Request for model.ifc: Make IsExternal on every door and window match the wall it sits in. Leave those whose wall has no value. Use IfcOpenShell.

First a look at what the model holds.

```python
import ifcopenshell
import ifcopenshell.util.element

model = ifcopenshell.open("model.ifc")
print(model.schema)
seen = {}
for e in model.by_type("IfcDoor") + model.by_type("IfcWindow"):
    if not e.FillsVoids:
        continue
    host = e.FillsVoids[0].RelatingOpeningElement.VoidsElements[0].RelatingBuildingElement
    own = ifcopenshell.util.element.get_pset(e, f"Pset_{e.is_a()[3:].removesuffix('StandardCase')}Common", "IsExternal")
    wall = ifcopenshell.util.element.get_pset(host, "Pset_WallCommon", "IsExternal")
    seen[e.is_a(), own, wall] = seen.get((e.is_a(), own, wall), 0) + 1
for (cls, own, wall), count in sorted(seen.items(), key=str):
    print(count, cls, "IsExternal:", own, "| host wall:", wall)
```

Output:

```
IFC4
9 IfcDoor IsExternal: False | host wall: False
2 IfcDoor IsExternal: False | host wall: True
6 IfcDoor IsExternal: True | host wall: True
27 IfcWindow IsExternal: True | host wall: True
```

```python
import ifcopenshell
import ifcopenshell.api.pset
import ifcopenshell.util.element

model = ifcopenshell.open("model.ifc")

count = 0
for ifc_class, pset_name in (("IfcDoor", "Pset_DoorCommon"), ("IfcWindow", "Pset_WindowCommon")):
    for e in model.by_type(ifc_class):
        if not e.FillsVoids:
            continue
        host = e.FillsVoids[0].RelatingOpeningElement.VoidsElements[0].RelatingBuildingElement
        external = ifcopenshell.util.element.get_pset(host, "Pset_WallCommon", "IsExternal")
        if external is None or ifcopenshell.util.element.get_pset(e, pset_name, "IsExternal") == external:
            continue
        pset = ifcopenshell.api.pset.add_pset(model, product=e, name=pset_name)
        ifcopenshell.api.pset.edit_pset(model, pset=pset, properties={"IsExternal": external})
        count += 1

print(count, "updated")

model.write("model_updated.ifc")
```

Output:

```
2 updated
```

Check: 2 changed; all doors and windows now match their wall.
